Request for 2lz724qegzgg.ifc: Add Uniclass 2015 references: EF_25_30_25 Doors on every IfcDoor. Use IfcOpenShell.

First a look at what the model holds.

```python
import ifcopenshell

model = ifcopenshell.open("2lz724qegzgg.ifc")
print(model.schema)
print("classifications:", [c.Name for c in model.by_type("IfcClassification")])
for ifc_class in ("IfcDoor", "IfcRoof", "IfcStair", "IfcWall", "IfcWindow"):
    print(ifc_class, len(model.by_type(ifc_class)))
```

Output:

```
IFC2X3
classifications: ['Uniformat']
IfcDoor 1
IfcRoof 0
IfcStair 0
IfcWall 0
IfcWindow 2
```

```python
import ifcopenshell
import ifcopenshell.api.classification

model = ifcopenshell.open("2lz724qegzgg.ifc")

# IFC2X3 requires Source and Edition and has no link from the project to the system.
system = model.create_entity("IfcClassification", Source="NBS", Edition="2015", Name="Uniclass 2015")

codes = {
    "IfcDoor": ("EF_25_30_25", "Doors"),
}
for ifc_class, (code, name) in codes.items():
    products = model.by_type(ifc_class)
    ifcopenshell.api.classification.add_reference(
        model, products=products, classification=system, identification=code, name=name
    )
    print(code, len(products))

model.write("2lz724qegzgg_edited.ifc")
```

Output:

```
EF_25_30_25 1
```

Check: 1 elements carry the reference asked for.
